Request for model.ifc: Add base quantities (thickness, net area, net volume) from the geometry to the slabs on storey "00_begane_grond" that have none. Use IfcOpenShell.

First a look at what the model holds.

```python
import ifcopenshell
import ifcopenshell.util.element
import ifcopenshell.util.unit

model = ifcopenshell.open("model.ifc")
print(model.schema)
for unit_type in ("LENGTHUNIT", "AREAUNIT", "VOLUMEUNIT"):
    print(unit_type, ifcopenshell.util.unit.calculate_unit_scale(model, unit_type))
storey = next(s for s in model.by_type("IfcBuildingStorey") if s.Name == "00_begane_grond")
slabs = [e for e in ifcopenshell.util.element.get_decomposition(storey) if e.is_a("IfcSlab")]
for e in sorted(slabs, key=lambda e: e.id()):
    print(e.id(), e.is_a(), e.Name, list(ifcopenshell.util.element.get_psets(e, qtos_only=True)), sep=" | ")
```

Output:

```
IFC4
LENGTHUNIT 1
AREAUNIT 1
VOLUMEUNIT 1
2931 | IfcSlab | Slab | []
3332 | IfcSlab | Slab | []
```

```python
import ifcopenshell
import ifcopenshell.api.pset
import ifcopenshell.geom
import ifcopenshell.util.element
import ifcopenshell.util.shape
import ifcopenshell.util.unit

model = ifcopenshell.open("model.ifc")
unit_scale = ifcopenshell.util.unit.calculate_unit_scale(model)
area_scale = ifcopenshell.util.unit.calculate_unit_scale(model, "AREAUNIT")
volume_scale = ifcopenshell.util.unit.calculate_unit_scale(model, "VOLUMEUNIT")
settings = ifcopenshell.geom.settings()

storey = next(s for s in model.by_type("IfcBuildingStorey") if s.Name == "00_begane_grond")
slabs = [e for e in ifcopenshell.util.element.get_decomposition(storey) if e.is_a("IfcSlab")]

for e in sorted(slabs, key=lambda e: e.id()):
    if ifcopenshell.util.element.get_psets(e, qtos_only=True, should_inherit=False):
        continue
    # Geometry comes back in metres, in the element's own axes.
    shape = ifcopenshell.geom.create_shape(settings, e)
    values = {
        "Width": ifcopenshell.util.shape.get_z(shape.geometry) / unit_scale,
        "NetArea": ifcopenshell.util.shape.get_footprint_area(shape.geometry) / area_scale,
        "NetVolume": ifcopenshell.util.shape.get_volume(shape.geometry) / volume_scale,
    }
    qto = ifcopenshell.api.pset.add_qto(model, product=e, name="Qto_SlabBaseQuantities")
    ifcopenshell.api.pset.edit_qto(model, qto=qto, properties=values)
    print(e.id(), {k: round(v, 3) for k, v in values.items()})

model.write("model_edited.ifc")
```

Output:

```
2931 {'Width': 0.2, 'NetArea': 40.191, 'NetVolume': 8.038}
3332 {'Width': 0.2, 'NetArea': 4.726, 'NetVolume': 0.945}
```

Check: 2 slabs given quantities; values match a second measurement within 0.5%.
